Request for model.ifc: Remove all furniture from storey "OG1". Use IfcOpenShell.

First a look at what the model holds.

```python
import ifcopenshell
import ifcopenshell.util.element

model = ifcopenshell.open("model.ifc")
print(model.schema)
storey = next(s for s in model.by_type("IfcBuildingStorey") if s.Name == "OG1")
furniture = [e for e in ifcopenshell.util.element.get_decomposition(storey) if e.is_a("IfcFurnishingElement")]
seen = {}
for e in furniture:
    element_type = ifcopenshell.util.element.get_type(e)
    name = element_type.Name if element_type not in (None, e) else None
    seen[name] = seen.get(name, 0) + 1
for name, count in sorted(seen.items(), key=str):
    print(count, "x", name)
```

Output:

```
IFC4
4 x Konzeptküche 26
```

```python
import ifcopenshell
import ifcopenshell.api.root
import ifcopenshell.util.element

model = ifcopenshell.open("model.ifc")

storey = next(s for s in model.by_type("IfcBuildingStorey") if s.Name == "OG1")
furniture = [e for e in ifcopenshell.util.element.get_decomposition(storey) if e.is_a("IfcFurnishingElement")]

for e in furniture:
    ifcopenshell.api.root.remove_product(model, product=e)
print(len(furniture), "removed")

model.write("model_edited.ifc")
```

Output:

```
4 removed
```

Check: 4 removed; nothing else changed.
